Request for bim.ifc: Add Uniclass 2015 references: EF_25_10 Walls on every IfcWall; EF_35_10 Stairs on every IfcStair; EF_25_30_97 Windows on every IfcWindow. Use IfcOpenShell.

First a look at what the model holds.

```python
import ifcopenshell

model = ifcopenshell.open("bim.ifc")
print(model.schema)
print("classifications:", [c.Name for c in model.by_type("IfcClassification")])
for ifc_class in ("IfcDoor", "IfcRoof", "IfcStair", "IfcWall", "IfcWindow"):
    print(ifc_class, len(model.by_type(ifc_class)))
```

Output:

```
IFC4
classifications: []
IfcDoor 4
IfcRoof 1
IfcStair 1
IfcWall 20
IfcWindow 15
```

```python
import ifcopenshell
import ifcopenshell.api.classification

model = ifcopenshell.open("bim.ifc")

system = ifcopenshell.api.classification.add_classification(model, classification="Uniclass 2015")

codes = {
    "IfcWall": ("EF_25_10", "Walls"),
    "IfcStair": ("EF_35_10", "Stairs"),
    "IfcWindow": ("EF_25_30_97", "Windows"),
}
for ifc_class, (code, name) in codes.items():
    products = model.by_type(ifc_class)
    ifcopenshell.api.classification.add_reference(
        model, products=products, classification=system, identification=code, name=name
    )
    print(code, len(products))

model.write("bim_v2.ifc")
```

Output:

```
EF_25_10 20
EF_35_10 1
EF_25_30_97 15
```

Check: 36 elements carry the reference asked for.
